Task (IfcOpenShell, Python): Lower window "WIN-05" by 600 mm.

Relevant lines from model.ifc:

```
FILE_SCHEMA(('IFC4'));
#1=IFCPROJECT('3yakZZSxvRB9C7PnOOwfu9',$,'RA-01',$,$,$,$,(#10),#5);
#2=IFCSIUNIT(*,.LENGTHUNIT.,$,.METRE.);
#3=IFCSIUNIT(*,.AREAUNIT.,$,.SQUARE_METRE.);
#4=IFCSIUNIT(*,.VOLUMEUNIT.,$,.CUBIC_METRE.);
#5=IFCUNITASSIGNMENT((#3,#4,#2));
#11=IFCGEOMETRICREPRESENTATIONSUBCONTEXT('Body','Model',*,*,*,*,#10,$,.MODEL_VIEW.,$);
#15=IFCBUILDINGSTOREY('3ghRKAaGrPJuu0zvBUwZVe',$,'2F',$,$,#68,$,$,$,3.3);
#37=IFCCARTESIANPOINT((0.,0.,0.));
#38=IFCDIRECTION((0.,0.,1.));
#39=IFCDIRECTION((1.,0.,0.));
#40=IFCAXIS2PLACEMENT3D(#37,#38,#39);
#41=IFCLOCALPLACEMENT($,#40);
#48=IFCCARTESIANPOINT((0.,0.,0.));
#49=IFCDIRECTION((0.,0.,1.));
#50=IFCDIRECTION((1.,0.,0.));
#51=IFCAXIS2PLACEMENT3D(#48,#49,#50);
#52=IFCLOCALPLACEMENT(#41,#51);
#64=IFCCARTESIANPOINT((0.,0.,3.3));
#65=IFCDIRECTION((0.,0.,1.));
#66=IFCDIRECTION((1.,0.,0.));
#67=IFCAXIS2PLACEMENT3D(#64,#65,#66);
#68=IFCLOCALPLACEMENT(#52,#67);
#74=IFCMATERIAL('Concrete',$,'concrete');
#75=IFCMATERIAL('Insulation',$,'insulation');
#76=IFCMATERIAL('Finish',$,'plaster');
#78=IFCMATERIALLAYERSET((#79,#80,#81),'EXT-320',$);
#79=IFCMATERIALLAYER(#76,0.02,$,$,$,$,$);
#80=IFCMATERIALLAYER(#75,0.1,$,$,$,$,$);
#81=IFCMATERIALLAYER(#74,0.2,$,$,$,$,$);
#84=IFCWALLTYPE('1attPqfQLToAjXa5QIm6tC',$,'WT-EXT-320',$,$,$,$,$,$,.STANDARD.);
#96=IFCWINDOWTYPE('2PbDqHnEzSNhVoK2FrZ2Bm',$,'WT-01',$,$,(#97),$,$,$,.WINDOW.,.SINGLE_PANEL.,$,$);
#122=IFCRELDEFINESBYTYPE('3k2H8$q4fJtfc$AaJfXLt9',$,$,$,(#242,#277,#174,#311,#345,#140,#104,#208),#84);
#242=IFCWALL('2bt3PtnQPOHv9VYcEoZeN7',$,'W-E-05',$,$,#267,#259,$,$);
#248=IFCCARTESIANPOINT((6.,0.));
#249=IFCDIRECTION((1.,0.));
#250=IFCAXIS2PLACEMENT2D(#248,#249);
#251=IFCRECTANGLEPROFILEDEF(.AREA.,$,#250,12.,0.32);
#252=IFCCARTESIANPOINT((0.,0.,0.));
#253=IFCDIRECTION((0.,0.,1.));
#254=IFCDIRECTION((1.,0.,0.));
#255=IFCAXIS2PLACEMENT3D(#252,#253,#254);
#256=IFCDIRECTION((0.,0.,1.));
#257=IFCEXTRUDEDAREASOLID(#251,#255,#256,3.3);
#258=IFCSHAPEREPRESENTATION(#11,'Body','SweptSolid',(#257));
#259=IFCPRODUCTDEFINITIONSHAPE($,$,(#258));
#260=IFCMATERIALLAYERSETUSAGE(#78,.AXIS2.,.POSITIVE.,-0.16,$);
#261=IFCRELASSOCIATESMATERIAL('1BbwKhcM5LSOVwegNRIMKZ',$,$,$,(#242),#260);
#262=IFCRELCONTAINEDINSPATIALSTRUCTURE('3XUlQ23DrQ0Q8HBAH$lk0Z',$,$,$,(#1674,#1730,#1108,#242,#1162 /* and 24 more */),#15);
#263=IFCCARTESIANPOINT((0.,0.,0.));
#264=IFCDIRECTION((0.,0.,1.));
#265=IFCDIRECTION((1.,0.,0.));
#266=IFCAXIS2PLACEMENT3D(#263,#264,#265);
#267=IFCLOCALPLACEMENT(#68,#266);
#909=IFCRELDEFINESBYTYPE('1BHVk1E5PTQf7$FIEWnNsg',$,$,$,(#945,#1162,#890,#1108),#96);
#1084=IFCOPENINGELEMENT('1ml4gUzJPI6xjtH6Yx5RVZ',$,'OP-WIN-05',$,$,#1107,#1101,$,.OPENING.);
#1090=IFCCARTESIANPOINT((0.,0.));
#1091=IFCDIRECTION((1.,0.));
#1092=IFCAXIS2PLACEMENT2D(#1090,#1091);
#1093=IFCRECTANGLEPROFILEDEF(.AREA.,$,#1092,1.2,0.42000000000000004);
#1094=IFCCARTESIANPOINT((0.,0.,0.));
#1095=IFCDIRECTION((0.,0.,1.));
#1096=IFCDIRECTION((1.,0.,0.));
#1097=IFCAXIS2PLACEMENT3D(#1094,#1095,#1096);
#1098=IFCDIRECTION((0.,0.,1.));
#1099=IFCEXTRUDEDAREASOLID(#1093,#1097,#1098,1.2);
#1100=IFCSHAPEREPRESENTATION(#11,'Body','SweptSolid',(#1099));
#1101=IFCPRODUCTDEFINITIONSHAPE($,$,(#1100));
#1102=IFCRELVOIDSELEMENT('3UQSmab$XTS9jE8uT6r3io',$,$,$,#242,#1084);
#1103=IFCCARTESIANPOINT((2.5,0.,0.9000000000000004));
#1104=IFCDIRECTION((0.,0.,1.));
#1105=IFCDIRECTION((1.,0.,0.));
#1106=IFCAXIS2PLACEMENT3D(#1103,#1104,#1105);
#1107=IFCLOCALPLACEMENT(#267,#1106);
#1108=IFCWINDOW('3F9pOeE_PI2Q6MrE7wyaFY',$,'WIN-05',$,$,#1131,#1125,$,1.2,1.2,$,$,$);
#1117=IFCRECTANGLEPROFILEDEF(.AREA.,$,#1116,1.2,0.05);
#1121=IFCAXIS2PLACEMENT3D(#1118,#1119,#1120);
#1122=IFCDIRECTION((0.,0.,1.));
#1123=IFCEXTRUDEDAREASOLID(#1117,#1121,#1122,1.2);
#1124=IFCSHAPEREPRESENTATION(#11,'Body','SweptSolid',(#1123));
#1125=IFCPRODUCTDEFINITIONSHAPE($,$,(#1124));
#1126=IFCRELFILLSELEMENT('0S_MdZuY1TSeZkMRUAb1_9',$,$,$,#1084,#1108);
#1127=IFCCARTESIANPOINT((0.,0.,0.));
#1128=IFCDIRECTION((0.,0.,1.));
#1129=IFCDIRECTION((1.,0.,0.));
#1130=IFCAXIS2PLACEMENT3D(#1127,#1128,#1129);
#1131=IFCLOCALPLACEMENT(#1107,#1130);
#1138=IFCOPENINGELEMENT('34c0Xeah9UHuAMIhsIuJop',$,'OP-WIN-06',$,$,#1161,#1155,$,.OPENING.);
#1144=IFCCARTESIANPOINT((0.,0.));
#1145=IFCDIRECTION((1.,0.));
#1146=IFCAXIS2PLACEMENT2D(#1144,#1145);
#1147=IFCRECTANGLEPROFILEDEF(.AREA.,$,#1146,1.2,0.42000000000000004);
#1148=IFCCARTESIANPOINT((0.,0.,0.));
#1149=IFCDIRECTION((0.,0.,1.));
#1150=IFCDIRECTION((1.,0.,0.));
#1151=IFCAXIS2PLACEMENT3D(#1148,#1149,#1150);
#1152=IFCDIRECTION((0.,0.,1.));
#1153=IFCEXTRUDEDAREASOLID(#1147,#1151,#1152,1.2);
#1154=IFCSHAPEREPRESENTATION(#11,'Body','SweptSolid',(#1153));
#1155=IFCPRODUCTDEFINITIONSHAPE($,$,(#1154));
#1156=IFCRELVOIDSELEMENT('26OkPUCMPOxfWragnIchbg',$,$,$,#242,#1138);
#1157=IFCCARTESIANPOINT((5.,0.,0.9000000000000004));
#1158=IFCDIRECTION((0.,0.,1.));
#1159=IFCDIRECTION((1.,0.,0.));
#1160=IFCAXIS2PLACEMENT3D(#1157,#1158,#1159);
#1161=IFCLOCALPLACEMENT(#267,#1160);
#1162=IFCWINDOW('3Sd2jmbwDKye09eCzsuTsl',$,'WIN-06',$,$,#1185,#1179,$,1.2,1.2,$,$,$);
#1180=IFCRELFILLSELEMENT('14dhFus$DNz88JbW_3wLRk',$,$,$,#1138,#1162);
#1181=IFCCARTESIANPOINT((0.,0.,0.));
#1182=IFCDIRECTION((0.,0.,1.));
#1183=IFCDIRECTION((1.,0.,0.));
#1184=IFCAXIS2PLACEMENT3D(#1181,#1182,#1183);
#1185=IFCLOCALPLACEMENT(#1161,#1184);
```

```python
import numpy as np
import ifcopenshell
import ifcopenshell.api.geometry
import ifcopenshell.util.placement
import ifcopenshell.util.unit

model = ifcopenshell.open("model.ifc")
unit_scale = ifcopenshell.util.unit.calculate_unit_scale(model)

window = model.by_id(1108)
opening = window.FillsVoids[0].RelatingOpeningElement
dz = -0.6 / unit_scale

shift = np.array([0.0, 0.0, dz])
# The window is placed relative to its opening, so it follows when the opening moves.
matrix = ifcopenshell.util.placement.get_local_placement(opening.ObjectPlacement)
matrix[:3, 3] += shift
ifcopenshell.api.geometry.edit_object_placement(
    model, product=opening, matrix=matrix, is_si=False, should_transform_children=True
)

print(f"moved by {dz * unit_scale:+.3f} m")

model.write("model_rev.ifc")
```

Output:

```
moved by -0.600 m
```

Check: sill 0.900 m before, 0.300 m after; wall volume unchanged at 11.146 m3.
